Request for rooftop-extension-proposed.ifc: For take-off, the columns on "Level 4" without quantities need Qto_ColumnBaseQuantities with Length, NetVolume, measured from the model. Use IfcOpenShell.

First a look at what the model holds.

```python
import ifcopenshell
import ifcopenshell.util.element
import ifcopenshell.util.unit

model = ifcopenshell.open("rooftop-extension-proposed.ifc")
print(model.schema)
for unit_type in ("LENGTHUNIT", "AREAUNIT", "VOLUMEUNIT"):
    print(unit_type, ifcopenshell.util.unit.calculate_unit_scale(model, unit_type))
storey = next(s for s in model.by_type("IfcBuildingStorey") if s.Name == "Level 4")
columns = [e for e in ifcopenshell.util.element.get_decomposition(storey) if e.is_a("IfcColumn")]
for e in sorted(columns, key=lambda e: e.id()):
    print(e.id(), e.is_a(), e.Name, list(ifcopenshell.util.element.get_psets(e, qtos_only=True)), sep=" | ")
```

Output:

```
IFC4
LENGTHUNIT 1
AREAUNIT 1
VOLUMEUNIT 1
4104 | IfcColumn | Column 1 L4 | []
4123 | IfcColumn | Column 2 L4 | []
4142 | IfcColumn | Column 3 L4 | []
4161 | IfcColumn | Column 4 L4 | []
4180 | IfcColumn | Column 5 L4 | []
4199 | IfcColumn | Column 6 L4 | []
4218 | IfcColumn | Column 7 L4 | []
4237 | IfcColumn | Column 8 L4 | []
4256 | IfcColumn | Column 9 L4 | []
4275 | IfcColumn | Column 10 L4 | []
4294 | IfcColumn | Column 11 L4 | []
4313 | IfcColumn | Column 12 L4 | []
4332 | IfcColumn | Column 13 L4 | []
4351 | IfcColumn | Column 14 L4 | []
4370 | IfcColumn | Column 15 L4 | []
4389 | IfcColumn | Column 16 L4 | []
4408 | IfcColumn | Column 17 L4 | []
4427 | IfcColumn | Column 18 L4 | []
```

```python
import ifcopenshell
import ifcopenshell.api.pset
import ifcopenshell.geom
import ifcopenshell.util.element
import ifcopenshell.util.shape
import ifcopenshell.util.unit

model = ifcopenshell.open("rooftop-extension-proposed.ifc")
unit_scale = ifcopenshell.util.unit.calculate_unit_scale(model)
volume_scale = ifcopenshell.util.unit.calculate_unit_scale(model, "VOLUMEUNIT")
settings = ifcopenshell.geom.settings()

storey = next(s for s in model.by_type("IfcBuildingStorey") if s.Name == "Level 4")
columns = [e for e in ifcopenshell.util.element.get_decomposition(storey) if e.is_a("IfcColumn")]

for e in sorted(columns, key=lambda e: e.id()):
    if ifcopenshell.util.element.get_psets(e, qtos_only=True, should_inherit=False):
        continue
    # Geometry comes back in metres, in the element's own axes.
    shape = ifcopenshell.geom.create_shape(settings, e)
    values = {
        "Length": ifcopenshell.util.shape.get_z(shape.geometry) / unit_scale,
        "NetVolume": ifcopenshell.util.shape.get_volume(shape.geometry) / volume_scale,
    }
    qto = ifcopenshell.api.pset.add_qto(model, product=e, name="Qto_ColumnBaseQuantities")
    ifcopenshell.api.pset.edit_qto(model, qto=qto, properties=values)
    print(e.id(), {k: round(v, 3) for k, v in values.items()})

model.write("rooftop-extension-proposed_v2.ifc")
```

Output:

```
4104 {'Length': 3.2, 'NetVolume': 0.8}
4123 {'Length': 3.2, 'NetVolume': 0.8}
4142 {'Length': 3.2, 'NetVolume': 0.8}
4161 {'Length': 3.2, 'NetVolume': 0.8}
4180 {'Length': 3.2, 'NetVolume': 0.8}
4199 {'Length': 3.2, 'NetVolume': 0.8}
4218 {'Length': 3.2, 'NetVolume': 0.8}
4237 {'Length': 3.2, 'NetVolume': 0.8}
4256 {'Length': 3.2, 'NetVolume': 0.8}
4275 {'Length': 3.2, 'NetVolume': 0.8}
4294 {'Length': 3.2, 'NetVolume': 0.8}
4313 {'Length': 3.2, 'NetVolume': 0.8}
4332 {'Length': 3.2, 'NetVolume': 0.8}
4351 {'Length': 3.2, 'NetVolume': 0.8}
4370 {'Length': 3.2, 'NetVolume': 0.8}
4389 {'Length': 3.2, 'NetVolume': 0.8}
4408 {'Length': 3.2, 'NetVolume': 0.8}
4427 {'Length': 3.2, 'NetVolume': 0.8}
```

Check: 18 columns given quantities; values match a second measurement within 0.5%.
